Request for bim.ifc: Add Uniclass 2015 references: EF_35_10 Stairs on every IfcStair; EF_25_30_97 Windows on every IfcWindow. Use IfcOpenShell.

First a look at what the model holds.

```python
import ifcopenshell

model = ifcopenshell.open("bim.ifc")
print(model.schema)
print("classifications:", [c.Name for c in model.by_type("IfcClassification")])
for ifc_class in ("IfcDoor", "IfcRoof", "IfcStair", "IfcWall", "IfcWindow"):
    print(ifc_class, len(model.by_type(ifc_class)))
```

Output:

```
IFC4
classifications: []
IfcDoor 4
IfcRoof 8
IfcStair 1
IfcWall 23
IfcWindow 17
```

```python
import ifcopenshell
import ifcopenshell.api.classification

model = ifcopenshell.open("bim.ifc")

system = ifcopenshell.api.classification.add_classification(model, classification="Uniclass 2015")

codes = {
    "IfcStair": ("EF_35_10", "Stairs"),
    "IfcWindow": ("EF_25_30_97", "Windows"),
}
for ifc_class, (code, name) in codes.items():
    products = model.by_type(ifc_class)
    ifcopenshell.api.classification.add_reference(
        model, products=products, classification=system, identification=code, name=name
    )
    print(code, len(products))

model.write("bim_edited.ifc")
```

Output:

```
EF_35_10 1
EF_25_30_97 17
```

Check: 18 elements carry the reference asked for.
